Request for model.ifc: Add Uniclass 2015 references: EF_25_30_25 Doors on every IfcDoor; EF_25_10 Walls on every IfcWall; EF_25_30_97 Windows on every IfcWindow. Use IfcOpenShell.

First a look at what the model holds.

```python
import ifcopenshell

model = ifcopenshell.open("model.ifc")
print(model.schema)
print("classifications:", [c.Name for c in model.by_type("IfcClassification")])
for ifc_class in ("IfcDoor", "IfcRoof", "IfcStair", "IfcWall", "IfcWindow"):
    print(ifc_class, len(model.by_type(ifc_class)))
```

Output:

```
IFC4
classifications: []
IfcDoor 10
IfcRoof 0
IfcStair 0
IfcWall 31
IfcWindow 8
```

```python
import ifcopenshell
import ifcopenshell.api.classification

model = ifcopenshell.open("model.ifc")

system = ifcopenshell.api.classification.add_classification(model, classification="Uniclass 2015")

codes = {
    "IfcDoor": ("EF_25_30_25", "Doors"),
    "IfcWall": ("EF_25_10", "Walls"),
    "IfcWindow": ("EF_25_30_97", "Windows"),
}
for ifc_class, (code, name) in codes.items():
    products = model.by_type(ifc_class)
    ifcopenshell.api.classification.add_reference(
        model, products=products, classification=system, identification=code, name=name
    )
    print(code, len(products))

model.write("model_v2.ifc")
```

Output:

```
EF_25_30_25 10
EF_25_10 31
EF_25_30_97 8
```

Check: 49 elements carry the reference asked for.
